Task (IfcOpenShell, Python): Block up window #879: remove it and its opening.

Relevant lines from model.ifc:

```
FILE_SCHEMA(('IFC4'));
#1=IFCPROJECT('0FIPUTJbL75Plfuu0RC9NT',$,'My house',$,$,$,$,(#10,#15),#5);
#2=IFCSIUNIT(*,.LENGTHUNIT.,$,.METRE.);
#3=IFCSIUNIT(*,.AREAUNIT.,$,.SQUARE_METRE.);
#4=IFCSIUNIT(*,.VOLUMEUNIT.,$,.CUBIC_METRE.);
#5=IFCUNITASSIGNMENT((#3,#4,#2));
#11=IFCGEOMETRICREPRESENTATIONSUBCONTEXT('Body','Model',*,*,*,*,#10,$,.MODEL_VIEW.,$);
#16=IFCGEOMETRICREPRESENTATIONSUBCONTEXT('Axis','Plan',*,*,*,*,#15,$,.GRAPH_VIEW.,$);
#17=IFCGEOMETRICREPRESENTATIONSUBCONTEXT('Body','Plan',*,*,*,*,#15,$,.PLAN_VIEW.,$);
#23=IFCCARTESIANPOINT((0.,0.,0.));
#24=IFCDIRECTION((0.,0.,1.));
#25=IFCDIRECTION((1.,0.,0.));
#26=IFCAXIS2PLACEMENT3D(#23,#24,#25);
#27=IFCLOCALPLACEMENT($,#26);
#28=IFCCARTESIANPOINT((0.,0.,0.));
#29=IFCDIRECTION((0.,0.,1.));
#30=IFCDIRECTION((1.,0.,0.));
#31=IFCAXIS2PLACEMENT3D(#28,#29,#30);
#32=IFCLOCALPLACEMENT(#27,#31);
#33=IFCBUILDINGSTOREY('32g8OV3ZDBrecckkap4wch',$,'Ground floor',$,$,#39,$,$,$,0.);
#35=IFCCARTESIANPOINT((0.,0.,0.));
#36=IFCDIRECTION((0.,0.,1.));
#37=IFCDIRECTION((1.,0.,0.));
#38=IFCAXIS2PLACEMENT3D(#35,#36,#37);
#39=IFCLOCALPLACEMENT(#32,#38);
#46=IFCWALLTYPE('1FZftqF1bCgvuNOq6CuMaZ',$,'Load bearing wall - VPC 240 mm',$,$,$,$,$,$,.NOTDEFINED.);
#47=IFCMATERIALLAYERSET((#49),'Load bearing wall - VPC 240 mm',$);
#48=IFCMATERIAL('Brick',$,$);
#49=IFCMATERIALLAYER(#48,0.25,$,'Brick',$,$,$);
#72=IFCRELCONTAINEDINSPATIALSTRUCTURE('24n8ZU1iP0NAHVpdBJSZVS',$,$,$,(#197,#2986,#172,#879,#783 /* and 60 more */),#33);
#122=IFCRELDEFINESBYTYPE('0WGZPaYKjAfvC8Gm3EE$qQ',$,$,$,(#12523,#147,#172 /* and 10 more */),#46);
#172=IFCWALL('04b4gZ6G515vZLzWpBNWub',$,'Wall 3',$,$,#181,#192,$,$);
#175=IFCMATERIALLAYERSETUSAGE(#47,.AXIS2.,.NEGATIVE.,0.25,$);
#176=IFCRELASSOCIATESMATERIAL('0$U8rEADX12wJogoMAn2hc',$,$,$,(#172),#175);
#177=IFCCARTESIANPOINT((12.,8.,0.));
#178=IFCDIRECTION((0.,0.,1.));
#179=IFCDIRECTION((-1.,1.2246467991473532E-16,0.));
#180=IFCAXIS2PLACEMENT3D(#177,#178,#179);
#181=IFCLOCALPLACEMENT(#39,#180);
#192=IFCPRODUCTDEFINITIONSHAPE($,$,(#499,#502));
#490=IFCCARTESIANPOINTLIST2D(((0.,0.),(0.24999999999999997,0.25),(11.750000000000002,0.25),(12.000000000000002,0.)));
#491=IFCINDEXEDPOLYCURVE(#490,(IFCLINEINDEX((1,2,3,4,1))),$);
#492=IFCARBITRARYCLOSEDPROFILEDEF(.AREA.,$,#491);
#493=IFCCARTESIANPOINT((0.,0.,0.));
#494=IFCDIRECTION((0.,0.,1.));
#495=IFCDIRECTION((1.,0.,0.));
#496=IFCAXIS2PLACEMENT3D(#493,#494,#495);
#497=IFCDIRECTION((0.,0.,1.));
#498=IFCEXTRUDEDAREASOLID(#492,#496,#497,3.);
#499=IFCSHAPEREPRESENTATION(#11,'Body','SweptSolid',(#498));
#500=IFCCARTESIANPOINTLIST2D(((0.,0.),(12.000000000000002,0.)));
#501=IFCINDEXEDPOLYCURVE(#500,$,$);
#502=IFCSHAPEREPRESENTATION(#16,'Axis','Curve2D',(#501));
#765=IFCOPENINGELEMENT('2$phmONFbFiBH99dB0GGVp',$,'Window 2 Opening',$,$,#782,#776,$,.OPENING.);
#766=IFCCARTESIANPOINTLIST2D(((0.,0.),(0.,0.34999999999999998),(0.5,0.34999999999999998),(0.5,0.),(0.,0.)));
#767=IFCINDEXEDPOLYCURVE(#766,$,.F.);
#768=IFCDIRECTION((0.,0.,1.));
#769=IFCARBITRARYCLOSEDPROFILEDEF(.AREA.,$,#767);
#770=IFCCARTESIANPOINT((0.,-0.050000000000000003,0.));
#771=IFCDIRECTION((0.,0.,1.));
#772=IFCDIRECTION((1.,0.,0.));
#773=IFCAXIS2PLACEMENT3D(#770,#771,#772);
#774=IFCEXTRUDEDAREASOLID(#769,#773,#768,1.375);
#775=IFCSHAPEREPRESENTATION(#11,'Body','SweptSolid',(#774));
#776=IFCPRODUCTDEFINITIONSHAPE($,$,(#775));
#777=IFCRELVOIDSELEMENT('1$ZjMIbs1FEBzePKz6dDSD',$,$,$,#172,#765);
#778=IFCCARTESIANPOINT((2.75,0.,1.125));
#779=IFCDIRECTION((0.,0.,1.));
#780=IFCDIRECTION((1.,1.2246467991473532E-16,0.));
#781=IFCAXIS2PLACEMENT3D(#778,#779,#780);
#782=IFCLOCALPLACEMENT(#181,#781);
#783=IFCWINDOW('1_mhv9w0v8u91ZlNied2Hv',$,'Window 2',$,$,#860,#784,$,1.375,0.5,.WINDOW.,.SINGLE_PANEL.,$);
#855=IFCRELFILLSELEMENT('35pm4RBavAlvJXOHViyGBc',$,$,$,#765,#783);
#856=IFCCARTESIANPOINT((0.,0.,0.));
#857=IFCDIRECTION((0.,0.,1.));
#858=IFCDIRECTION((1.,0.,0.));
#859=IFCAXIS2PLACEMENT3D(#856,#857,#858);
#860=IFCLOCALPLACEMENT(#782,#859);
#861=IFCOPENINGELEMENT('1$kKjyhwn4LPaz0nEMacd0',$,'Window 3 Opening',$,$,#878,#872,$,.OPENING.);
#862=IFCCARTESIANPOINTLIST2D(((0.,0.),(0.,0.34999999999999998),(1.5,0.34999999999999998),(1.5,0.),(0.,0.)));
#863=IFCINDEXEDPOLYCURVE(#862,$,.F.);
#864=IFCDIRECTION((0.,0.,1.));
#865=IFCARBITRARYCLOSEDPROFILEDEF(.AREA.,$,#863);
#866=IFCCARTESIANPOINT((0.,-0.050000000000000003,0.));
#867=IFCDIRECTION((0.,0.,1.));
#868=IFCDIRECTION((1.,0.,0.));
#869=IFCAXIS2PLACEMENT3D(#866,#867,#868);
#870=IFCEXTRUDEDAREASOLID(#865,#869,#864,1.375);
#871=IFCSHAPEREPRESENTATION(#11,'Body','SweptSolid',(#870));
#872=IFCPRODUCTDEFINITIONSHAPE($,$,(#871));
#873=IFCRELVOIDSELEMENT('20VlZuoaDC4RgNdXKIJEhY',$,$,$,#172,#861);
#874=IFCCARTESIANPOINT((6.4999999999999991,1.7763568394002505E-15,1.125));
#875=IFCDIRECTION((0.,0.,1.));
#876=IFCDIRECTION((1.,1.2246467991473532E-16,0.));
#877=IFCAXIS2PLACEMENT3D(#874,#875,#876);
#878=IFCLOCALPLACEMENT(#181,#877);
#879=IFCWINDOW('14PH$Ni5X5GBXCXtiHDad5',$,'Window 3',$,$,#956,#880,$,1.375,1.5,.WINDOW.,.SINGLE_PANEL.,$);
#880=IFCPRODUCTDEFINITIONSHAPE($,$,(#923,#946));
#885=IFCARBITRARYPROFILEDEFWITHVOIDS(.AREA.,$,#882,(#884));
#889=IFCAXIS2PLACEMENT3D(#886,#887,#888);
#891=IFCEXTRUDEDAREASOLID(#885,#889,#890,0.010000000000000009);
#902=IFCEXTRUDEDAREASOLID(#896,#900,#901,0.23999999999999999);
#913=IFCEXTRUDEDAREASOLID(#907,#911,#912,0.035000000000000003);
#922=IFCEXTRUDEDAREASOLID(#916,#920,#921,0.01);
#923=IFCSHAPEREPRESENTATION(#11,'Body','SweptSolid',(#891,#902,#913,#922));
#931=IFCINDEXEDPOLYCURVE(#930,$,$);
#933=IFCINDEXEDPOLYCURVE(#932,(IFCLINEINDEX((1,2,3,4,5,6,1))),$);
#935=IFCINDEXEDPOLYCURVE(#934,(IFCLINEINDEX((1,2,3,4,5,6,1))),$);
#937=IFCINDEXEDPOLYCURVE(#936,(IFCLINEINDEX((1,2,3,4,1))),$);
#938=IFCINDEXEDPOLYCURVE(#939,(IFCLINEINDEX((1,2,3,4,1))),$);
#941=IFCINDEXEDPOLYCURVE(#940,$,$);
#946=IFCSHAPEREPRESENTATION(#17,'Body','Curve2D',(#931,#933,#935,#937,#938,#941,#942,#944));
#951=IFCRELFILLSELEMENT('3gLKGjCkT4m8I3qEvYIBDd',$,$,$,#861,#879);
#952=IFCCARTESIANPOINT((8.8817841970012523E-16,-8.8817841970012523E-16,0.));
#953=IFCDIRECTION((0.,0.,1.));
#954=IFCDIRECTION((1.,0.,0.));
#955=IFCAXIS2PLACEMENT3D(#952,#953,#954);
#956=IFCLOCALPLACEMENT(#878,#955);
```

```python
import ifcopenshell
import ifcopenshell.api.feature
import ifcopenshell.api.root
import ifcopenshell.geom
import ifcopenshell.util.shape

model = ifcopenshell.open("model.ifc")
settings = ifcopenshell.geom.settings()


def volume(element):
    """Net volume in cubic metres, openings subtracted."""
    shape = ifcopenshell.geom.create_shape(settings, element)
    return ifcopenshell.util.shape.get_volume(shape.geometry)


window = model.by_guid("14PH$Ni5X5GBXCXtiHDad5")
opening = window.FillsVoids[0].RelatingOpeningElement
wall = opening.VoidsElements[0].RelatingBuildingElement
before = volume(wall)

ifcopenshell.api.root.remove_product(model, product=window)
ifcopenshell.api.feature.remove_feature(model, feature=opening)

after = volume(wall)

print(f"wall volume {before:.3f} -> {after:.3f} m3")

model.write("model_updated.ifc")
```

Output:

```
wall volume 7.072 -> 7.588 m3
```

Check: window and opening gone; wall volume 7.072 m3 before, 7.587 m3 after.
